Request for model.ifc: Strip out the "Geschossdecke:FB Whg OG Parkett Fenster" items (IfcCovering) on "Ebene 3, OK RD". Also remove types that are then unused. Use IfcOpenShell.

First a look at what the model holds.

```python
import ifcopenshell
import ifcopenshell.util.element

model = ifcopenshell.open("model.ifc")
print(model.schema)
storey = next(s for s in model.by_type("IfcBuildingStorey") if s.Name == "Ebene 3, OK RD")
coverings = [e for e in ifcopenshell.util.element.get_decomposition(storey) if e.is_a("IfcCovering")]
seen = {}
for e in coverings:
    element_type = ifcopenshell.util.element.get_type(e)
    name = element_type.Name if element_type not in (None, e) else None
    seen[name] = seen.get(name, 0) + 1
for name, count in sorted(seen.items(), key=str):
    print(count, "x", name)
```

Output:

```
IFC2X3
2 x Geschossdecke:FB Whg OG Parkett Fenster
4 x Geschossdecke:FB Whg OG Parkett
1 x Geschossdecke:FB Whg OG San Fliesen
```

```python
import ifcopenshell
import ifcopenshell.api.root
import ifcopenshell.util.element

model = ifcopenshell.open("model.ifc")

storey = next(s for s in model.by_type("IfcBuildingStorey") if s.Name == "Ebene 3, OK RD")
coverings = [e for e in ifcopenshell.util.element.get_decomposition(storey) if e.is_a("IfcCovering")]
targets = [e for e in coverings if (t := ifcopenshell.util.element.get_type(e)) not in (None, e) and t.Name == "Geschossdecke:FB Whg OG Parkett Fenster"]
types = {ifcopenshell.util.element.get_type(e) for e in targets} - {None, *targets}

for e in targets:
    ifcopenshell.api.root.remove_product(model, product=e)
print(len(targets), "removed")

unused = [t for t in types if not ifcopenshell.util.element.get_types(t)]
for t in unused:
    ifcopenshell.api.root.remove_product(model, product=t)
print(len(unused), "unused types removed")

model.write("model_v2.ifc")
```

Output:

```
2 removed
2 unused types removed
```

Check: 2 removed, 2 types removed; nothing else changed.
